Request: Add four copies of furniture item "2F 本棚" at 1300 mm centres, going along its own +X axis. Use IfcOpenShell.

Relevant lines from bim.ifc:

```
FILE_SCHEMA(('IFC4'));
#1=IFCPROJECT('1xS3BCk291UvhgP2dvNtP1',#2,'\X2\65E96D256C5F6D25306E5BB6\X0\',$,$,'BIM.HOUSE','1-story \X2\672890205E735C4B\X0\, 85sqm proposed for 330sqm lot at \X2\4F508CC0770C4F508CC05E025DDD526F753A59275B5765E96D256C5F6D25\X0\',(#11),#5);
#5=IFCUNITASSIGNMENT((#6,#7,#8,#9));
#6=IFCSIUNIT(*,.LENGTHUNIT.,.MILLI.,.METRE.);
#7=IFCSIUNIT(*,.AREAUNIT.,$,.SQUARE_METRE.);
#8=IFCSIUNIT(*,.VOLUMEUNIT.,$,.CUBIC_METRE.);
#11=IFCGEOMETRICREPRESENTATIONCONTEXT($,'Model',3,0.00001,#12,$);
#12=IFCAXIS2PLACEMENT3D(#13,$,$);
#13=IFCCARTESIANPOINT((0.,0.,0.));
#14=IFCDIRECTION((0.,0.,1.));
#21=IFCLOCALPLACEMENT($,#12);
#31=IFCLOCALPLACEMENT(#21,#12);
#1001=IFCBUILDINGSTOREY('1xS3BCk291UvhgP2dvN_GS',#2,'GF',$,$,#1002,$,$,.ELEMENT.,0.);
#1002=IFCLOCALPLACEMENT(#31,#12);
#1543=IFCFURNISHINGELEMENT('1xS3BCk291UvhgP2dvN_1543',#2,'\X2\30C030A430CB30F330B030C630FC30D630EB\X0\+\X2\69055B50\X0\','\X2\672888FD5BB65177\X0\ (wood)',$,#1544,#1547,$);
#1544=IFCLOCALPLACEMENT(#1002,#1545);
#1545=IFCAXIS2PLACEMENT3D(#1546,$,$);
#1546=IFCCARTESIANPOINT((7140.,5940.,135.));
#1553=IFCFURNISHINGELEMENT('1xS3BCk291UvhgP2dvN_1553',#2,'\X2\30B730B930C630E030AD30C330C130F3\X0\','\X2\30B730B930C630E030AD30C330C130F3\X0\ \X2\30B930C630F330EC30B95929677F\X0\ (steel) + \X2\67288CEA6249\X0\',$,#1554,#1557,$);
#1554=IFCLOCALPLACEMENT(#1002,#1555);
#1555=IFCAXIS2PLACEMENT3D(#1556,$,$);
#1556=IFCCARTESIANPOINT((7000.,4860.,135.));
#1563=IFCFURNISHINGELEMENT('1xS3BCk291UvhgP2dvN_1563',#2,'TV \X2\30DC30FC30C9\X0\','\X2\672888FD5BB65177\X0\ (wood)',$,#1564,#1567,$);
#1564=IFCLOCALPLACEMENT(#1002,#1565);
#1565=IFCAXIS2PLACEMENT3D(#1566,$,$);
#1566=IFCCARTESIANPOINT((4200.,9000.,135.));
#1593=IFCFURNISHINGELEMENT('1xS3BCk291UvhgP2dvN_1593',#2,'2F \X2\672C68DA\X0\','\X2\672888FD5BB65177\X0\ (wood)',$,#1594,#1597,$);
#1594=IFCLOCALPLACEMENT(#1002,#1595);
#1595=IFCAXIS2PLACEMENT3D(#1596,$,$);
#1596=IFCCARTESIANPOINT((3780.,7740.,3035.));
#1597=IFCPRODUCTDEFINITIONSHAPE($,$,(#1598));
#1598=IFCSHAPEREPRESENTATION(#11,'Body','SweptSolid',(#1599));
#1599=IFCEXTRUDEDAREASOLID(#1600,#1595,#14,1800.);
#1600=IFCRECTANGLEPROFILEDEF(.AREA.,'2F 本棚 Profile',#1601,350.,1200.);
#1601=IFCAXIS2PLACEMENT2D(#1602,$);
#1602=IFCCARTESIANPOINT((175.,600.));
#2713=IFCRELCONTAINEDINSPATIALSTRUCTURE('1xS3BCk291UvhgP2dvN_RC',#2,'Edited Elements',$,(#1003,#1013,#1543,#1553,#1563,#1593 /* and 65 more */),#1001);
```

```python
import ifcopenshell
import ifcopenshell.api.geometry
import ifcopenshell.api.root
import ifcopenshell.util.element
import ifcopenshell.util.placement

model = ifcopenshell.open("bim.ifc")


def reuse_history(source, copy):
    """copy_class also copies each property set's owner history, people and application; keep the originals."""
    for rel in copy.IsDefinedBy:
        if rel.is_a("IfcRelDefinesByProperties") and (history := rel.RelatingPropertyDefinition.OwnerHistory):
            rel.RelatingPropertyDefinition.OwnerHistory = source.OwnerHistory
            ifcopenshell.util.element.remove_deep2(model, history)


source = model.by_guid("1xS3BCk291UvhgP2dvN_1593")
base = ifcopenshell.util.placement.get_local_placement(source.ObjectPlacement)
step = base[:3, 0] * 1300.0

for i in range(1, 5):
    copy = ifcopenshell.api.root.copy_class(model, product=source)
    copy.Representation = ifcopenshell.util.element.copy_deep(
        model, source.Representation, exclude=["IfcGeometricRepresentationContext", "IfcRepresentationMap"]
    )
    reuse_history(source, copy)
    matrix = base.copy()
    matrix[:3, 3] += i * step
    print("added at", matrix[:3, 3].round(3) + 0.0)
    ifcopenshell.api.geometry.edit_object_placement(model, product=copy, matrix=matrix, is_si=False)

model.write("bim_edited.ifc")
```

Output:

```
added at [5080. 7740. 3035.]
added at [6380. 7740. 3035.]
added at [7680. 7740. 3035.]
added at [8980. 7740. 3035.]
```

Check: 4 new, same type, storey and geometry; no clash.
